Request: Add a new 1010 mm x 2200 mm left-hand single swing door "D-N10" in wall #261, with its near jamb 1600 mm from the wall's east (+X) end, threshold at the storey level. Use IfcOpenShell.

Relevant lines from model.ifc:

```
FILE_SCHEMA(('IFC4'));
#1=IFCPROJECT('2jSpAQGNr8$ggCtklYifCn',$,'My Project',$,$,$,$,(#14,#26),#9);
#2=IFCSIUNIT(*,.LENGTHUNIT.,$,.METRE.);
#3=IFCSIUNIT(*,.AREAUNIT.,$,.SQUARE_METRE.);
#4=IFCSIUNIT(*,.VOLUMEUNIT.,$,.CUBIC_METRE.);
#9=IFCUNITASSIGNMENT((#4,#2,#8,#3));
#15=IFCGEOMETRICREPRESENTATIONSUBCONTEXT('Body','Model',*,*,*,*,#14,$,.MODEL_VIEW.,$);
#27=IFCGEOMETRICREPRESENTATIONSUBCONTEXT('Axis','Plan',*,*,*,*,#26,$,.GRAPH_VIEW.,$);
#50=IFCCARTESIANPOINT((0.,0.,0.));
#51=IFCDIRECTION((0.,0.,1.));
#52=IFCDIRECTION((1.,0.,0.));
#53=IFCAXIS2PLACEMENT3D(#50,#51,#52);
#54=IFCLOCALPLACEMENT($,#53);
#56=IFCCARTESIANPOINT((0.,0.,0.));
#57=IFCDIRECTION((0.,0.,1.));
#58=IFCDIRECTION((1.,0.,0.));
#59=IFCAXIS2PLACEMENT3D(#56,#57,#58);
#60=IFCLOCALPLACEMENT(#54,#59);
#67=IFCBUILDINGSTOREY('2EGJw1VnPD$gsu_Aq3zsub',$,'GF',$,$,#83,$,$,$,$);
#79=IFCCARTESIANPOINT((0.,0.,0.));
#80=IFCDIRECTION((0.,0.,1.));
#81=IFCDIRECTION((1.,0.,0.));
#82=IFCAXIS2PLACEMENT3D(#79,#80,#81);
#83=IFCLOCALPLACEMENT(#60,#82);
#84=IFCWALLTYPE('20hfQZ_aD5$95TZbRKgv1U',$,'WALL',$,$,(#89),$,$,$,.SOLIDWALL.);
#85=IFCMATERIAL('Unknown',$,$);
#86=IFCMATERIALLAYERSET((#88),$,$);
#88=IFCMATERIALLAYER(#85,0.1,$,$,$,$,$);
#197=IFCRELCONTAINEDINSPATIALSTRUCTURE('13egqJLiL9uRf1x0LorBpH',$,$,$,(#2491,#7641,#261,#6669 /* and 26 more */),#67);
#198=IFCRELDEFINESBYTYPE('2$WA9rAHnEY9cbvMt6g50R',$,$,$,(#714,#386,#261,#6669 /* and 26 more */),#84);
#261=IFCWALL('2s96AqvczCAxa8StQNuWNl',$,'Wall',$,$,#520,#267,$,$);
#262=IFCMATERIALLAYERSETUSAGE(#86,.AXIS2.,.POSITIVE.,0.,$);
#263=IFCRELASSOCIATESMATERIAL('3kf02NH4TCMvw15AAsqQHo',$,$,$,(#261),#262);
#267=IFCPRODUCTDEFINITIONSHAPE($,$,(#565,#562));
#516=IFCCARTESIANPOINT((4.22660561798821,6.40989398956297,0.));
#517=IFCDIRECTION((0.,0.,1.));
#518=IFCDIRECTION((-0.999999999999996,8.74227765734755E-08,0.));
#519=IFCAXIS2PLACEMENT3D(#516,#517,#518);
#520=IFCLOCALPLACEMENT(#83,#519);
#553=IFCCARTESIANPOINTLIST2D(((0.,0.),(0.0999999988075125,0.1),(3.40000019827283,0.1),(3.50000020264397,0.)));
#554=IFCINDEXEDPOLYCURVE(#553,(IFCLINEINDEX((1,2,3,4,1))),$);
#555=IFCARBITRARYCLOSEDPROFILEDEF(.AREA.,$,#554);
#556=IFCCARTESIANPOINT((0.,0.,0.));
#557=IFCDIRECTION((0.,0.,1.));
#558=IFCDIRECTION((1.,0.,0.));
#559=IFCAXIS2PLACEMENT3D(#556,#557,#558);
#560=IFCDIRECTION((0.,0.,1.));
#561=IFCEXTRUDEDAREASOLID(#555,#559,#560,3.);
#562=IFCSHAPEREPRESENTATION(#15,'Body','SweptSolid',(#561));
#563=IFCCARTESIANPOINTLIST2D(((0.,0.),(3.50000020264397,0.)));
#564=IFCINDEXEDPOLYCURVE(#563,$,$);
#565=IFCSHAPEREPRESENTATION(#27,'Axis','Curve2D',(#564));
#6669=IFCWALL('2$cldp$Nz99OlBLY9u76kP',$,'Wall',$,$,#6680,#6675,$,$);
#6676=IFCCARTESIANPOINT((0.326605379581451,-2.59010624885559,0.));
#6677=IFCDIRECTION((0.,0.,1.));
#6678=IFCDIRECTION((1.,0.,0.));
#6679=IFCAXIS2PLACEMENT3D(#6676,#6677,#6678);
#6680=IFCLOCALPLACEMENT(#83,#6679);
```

```python
import numpy as np
import ifcopenshell
import ifcopenshell.api.feature
import ifcopenshell.api.geometry
import ifcopenshell.api.root
import ifcopenshell.api.spatial
import ifcopenshell.geom
import ifcopenshell.util.element
import ifcopenshell.util.placement
import ifcopenshell.util.representation
import ifcopenshell.util.shape
import ifcopenshell.util.unit

model = ifcopenshell.open("model.ifc")
unit_scale = ifcopenshell.util.unit.calculate_unit_scale(model)
settings = ifcopenshell.geom.settings()


def volume(element):
    """Net volume in cubic metres, openings subtracted."""
    shape = ifcopenshell.geom.create_shape(settings, element)
    return ifcopenshell.util.shape.get_volume(shape.geometry)


wall = model.by_guid("2s96AqvczCAxa8StQNuWNl")
storey = ifcopenshell.util.element.get_container(wall, ifc_class="IfcBuildingStorey")
context = ifcopenshell.util.representation.get_context(model, "Model", "Body", "MODEL_VIEW")
before = volume(wall)

width, height, from_end, sill = 1.01, 2.2, 1.6, 0.0  # metres

# The wall runs along its own X axis, and the end named is its -X end.
wall_shape = ifcopenshell.geom.create_shape(settings, wall)
x, y, z = ifcopenshell.util.shape.get_vertices(wall_shape.geometry).T
start = x.min() + from_end
face, thickness = float(y.min()), float(y.max() - y.min())
wall_matrix = ifcopenshell.util.placement.get_local_placement(wall.ObjectPlacement)
level = ifcopenshell.util.placement.get_local_placement(storey.ObjectPlacement)[2, 3]


def in_wall(x, y):
    """Placement at x, y metres in the wall's axes, at sill height."""
    matrix = wall_matrix.copy()
    matrix[:, 3] = wall_matrix @ np.array([x / unit_scale, y / unit_scale, 0.0, 1.0])
    matrix[2, 3] = level + sill / unit_scale
    return matrix


# Opening: a box that overshoots both wall faces by 50 mm.
opening = ifcopenshell.api.root.create_entity(model, ifc_class="IfcOpeningElement", predefined_type="OPENING")
box = ifcopenshell.api.geometry.add_wall_representation(
    model, context=context, length=width, height=height, thickness=thickness + 0.1
)
ifcopenshell.api.geometry.assign_representation(model, product=opening, representation=box)
ifcopenshell.api.geometry.edit_object_placement(model, product=opening, matrix=in_wall(start, face - 0.05), is_si=False)
ifcopenshell.api.feature.add_feature(model, feature=opening, element=wall)

door = ifcopenshell.api.root.create_entity(model, ifc_class="IfcDoor", name="D-N10", predefined_type="DOOR")
door.OverallWidth, door.OverallHeight = width / unit_scale, height / unit_scale
door.OperationType = "SINGLE_SWING_LEFT"
body = ifcopenshell.api.geometry.add_door_representation(
    model,
    context=context,
    overall_width=door.OverallWidth,
    overall_height=door.OverallHeight,
    operation_type="SINGLE_SWING_LEFT",
    lining_properties={"LiningDepth": thickness / unit_scale, "ThresholdDepth": thickness / unit_scale},
)
ifcopenshell.api.geometry.assign_representation(model, product=door, representation=body)
ifcopenshell.api.spatial.assign_container(model, products=[door], relating_structure=storey)
ifcopenshell.api.feature.add_filling(model, opening=opening, element=door)

# The lining spans the wall, so the door starts at the wall face.
ifcopenshell.api.geometry.edit_object_placement(model, product=door, matrix=in_wall(start, face), is_si=False)

after = volume(wall)

print(f"wall volume {before:.3f} -> {after:.3f} m3")

model.write("model_v2.ifc")
```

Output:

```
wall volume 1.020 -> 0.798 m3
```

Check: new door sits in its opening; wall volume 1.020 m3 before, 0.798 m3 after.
